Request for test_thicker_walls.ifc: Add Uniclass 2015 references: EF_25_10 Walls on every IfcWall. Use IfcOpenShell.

First a look at what the model holds.

```python
import ifcopenshell

model = ifcopenshell.open("test_thicker_walls.ifc")
print(model.schema)
print("classifications:", [c.Name for c in model.by_type("IfcClassification")])
for ifc_class in ("IfcDoor", "IfcRoof", "IfcStair", "IfcWall", "IfcWindow"):
    print(ifc_class, len(model.by_type(ifc_class)))
```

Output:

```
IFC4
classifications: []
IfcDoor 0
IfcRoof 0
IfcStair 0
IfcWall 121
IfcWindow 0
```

```python
import ifcopenshell
import ifcopenshell.api.classification

model = ifcopenshell.open("test_thicker_walls.ifc")

system = ifcopenshell.api.classification.add_classification(model, classification="Uniclass 2015")

codes = {
    "IfcWall": ("EF_25_10", "Walls"),
}
for ifc_class, (code, name) in codes.items():
    products = model.by_type(ifc_class)
    ifcopenshell.api.classification.add_reference(
        model, products=products, classification=system, identification=code, name=name
    )
    print(code, len(products))

model.write("test_thicker_walls_v2.ifc")
```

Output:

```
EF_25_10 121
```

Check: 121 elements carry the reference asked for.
